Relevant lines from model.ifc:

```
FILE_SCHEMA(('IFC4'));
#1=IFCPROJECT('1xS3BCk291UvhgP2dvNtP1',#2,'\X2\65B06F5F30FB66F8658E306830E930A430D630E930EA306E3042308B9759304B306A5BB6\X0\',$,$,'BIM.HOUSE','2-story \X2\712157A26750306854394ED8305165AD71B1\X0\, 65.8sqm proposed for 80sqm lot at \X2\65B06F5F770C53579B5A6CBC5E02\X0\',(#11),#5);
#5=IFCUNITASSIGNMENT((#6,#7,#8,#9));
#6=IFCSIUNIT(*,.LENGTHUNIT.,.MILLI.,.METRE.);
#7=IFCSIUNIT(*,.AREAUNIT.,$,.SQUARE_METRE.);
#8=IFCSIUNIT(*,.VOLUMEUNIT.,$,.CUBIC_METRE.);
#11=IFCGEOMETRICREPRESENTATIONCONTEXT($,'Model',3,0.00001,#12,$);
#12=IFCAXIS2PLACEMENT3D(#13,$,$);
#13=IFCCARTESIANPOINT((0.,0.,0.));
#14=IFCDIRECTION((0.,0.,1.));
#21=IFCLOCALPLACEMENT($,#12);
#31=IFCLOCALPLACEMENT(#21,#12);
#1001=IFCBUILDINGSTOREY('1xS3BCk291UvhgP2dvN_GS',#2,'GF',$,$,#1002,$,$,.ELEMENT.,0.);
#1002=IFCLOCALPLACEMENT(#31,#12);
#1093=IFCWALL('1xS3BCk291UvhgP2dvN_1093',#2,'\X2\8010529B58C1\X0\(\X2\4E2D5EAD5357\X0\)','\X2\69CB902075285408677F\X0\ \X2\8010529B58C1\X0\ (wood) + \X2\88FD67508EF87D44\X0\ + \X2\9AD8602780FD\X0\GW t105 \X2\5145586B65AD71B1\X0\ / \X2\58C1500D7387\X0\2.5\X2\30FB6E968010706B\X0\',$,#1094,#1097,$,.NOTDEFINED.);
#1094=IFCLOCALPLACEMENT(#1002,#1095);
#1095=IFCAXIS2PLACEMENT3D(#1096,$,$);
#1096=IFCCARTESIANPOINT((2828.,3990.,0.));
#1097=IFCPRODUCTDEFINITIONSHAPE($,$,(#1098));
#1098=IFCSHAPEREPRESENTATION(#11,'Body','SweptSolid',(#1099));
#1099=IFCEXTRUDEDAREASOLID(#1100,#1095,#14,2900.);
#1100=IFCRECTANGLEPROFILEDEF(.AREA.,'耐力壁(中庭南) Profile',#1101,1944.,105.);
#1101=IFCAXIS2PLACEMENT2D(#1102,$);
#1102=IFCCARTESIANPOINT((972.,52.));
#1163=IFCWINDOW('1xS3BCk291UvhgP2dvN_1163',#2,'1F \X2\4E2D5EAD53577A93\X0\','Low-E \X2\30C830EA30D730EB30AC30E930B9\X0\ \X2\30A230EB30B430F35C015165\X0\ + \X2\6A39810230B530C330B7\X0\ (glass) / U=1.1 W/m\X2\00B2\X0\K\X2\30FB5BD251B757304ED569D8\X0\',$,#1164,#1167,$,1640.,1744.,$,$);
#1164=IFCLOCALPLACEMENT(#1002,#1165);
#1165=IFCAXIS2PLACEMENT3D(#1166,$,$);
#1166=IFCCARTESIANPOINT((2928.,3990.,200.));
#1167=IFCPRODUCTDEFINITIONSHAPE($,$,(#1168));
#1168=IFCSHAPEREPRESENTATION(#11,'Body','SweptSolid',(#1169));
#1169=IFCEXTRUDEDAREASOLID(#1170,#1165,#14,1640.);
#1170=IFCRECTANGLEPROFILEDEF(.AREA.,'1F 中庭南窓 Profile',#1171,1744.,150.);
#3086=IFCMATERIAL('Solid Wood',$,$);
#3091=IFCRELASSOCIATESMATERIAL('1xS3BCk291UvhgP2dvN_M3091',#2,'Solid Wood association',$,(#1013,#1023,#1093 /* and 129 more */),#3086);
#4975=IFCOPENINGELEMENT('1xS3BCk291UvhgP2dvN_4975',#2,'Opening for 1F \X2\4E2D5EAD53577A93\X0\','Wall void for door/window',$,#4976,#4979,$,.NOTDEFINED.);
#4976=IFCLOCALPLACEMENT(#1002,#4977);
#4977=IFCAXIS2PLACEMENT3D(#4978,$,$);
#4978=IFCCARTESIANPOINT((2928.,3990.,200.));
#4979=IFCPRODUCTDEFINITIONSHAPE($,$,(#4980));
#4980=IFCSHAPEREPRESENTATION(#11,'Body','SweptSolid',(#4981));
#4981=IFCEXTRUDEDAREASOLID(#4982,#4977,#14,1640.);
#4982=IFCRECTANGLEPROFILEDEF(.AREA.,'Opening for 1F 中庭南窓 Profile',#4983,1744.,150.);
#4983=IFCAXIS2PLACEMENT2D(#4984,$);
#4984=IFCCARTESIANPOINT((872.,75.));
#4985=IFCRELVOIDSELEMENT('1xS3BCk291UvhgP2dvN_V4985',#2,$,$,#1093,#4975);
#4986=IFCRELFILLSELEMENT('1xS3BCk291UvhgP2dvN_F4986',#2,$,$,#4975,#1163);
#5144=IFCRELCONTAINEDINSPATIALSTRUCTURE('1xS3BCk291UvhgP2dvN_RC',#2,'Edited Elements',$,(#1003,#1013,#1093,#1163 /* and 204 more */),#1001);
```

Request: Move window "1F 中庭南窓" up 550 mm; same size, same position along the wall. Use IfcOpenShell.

```python
import numpy as np
import ifcopenshell
import ifcopenshell.api.geometry
import ifcopenshell.util.placement
import ifcopenshell.util.unit

model = ifcopenshell.open("model.ifc")
unit_scale = ifcopenshell.util.unit.calculate_unit_scale(model)

window = model.by_guid("1xS3BCk291UvhgP2dvN_1163")
opening = window.FillsVoids[0].RelatingOpeningElement
dz = 0.55 / unit_scale

shift = np.array([0.0, 0.0, dz])
# The window is not placed relative to its opening, so move both.
for product in (opening, window):
    matrix = ifcopenshell.util.placement.get_local_placement(product.ObjectPlacement)
    matrix[:3, 3] += shift
    ifcopenshell.api.geometry.edit_object_placement(model, product=product, matrix=matrix, is_si=False)

print(f"moved by {dz * unit_scale:+.3f} m")

model.write("model_rev.ifc")
```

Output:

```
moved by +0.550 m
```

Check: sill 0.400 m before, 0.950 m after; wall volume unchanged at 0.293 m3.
